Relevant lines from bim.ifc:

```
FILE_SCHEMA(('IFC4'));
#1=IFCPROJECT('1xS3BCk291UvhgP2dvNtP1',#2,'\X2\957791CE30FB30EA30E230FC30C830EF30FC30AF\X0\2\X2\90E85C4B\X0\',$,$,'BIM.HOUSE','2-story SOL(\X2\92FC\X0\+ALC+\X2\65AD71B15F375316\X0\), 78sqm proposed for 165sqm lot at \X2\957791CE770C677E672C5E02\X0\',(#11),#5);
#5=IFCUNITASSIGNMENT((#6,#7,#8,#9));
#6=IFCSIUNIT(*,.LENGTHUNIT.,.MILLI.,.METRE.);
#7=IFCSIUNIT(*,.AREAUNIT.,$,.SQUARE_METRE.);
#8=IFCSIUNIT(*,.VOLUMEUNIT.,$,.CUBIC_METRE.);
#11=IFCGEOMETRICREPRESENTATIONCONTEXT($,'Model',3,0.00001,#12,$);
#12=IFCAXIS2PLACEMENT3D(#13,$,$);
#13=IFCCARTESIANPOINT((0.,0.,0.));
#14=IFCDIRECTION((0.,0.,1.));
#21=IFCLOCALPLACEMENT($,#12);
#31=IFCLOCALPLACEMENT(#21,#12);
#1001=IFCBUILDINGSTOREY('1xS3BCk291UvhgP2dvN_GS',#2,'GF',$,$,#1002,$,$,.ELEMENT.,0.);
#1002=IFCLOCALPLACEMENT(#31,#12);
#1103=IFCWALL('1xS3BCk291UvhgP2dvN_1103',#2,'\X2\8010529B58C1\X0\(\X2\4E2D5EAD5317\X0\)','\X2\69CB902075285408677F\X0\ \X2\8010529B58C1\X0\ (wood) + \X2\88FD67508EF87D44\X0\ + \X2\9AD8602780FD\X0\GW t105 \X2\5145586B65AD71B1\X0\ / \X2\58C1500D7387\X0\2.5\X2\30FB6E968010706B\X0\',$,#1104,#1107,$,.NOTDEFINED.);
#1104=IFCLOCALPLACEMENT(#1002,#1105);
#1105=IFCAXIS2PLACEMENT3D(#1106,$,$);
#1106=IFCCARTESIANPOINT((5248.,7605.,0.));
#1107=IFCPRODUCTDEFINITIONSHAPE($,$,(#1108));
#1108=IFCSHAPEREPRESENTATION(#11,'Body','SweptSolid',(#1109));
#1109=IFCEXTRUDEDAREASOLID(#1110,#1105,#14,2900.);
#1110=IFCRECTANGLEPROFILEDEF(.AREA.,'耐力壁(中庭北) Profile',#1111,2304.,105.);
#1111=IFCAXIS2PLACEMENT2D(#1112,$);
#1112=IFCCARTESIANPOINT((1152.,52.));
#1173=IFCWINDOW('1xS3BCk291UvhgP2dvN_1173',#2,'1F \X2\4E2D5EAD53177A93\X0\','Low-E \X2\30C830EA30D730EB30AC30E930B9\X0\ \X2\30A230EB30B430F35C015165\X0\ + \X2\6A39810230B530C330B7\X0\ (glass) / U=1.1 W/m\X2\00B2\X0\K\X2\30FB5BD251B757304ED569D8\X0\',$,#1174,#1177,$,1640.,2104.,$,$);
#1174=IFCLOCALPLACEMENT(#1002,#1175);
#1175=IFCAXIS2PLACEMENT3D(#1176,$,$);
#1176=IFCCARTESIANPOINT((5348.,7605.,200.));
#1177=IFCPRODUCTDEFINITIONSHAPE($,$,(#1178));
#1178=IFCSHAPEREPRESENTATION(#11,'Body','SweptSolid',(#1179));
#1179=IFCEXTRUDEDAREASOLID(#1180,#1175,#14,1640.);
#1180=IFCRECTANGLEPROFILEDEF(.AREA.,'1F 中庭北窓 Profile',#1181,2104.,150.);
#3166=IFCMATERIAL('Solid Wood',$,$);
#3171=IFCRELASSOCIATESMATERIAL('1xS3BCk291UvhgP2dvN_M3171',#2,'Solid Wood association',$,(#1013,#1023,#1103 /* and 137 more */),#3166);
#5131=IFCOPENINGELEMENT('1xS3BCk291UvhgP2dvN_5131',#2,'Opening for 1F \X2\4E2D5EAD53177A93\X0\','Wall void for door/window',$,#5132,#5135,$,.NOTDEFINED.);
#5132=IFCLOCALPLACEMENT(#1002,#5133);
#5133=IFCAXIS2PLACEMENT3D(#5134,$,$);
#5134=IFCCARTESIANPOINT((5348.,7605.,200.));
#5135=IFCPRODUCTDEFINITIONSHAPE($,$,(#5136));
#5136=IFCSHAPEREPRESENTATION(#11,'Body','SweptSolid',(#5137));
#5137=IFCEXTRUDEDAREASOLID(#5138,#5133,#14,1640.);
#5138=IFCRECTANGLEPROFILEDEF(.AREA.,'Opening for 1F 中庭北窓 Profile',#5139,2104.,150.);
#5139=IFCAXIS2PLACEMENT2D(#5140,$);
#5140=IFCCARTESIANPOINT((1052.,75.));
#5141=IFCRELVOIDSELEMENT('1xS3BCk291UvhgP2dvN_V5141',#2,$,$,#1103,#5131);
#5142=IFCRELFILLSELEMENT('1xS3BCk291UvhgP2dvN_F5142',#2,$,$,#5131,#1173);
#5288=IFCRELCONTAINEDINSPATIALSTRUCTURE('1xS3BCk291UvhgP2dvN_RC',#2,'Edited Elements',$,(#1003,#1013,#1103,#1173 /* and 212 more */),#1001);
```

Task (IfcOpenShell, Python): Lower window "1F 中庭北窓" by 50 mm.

```python
import numpy as np
import ifcopenshell
import ifcopenshell.api.geometry
import ifcopenshell.util.placement
import ifcopenshell.util.unit

model = ifcopenshell.open("bim.ifc")
unit_scale = ifcopenshell.util.unit.calculate_unit_scale(model)

window = model.by_guid("1xS3BCk291UvhgP2dvN_1173")
opening = window.FillsVoids[0].RelatingOpeningElement
dz = -0.05 / unit_scale

shift = np.array([0.0, 0.0, dz])
# The window is not placed relative to its opening, so move both.
for product in (opening, window):
    matrix = ifcopenshell.util.placement.get_local_placement(product.ObjectPlacement)
    matrix[:3, 3] += shift
    ifcopenshell.api.geometry.edit_object_placement(model, product=product, matrix=matrix, is_si=False)

print(f"moved by {dz * unit_scale:+.3f} m")

model.write("bim_v2.ifc")
```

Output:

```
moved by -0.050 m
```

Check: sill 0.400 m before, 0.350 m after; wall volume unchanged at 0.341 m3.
